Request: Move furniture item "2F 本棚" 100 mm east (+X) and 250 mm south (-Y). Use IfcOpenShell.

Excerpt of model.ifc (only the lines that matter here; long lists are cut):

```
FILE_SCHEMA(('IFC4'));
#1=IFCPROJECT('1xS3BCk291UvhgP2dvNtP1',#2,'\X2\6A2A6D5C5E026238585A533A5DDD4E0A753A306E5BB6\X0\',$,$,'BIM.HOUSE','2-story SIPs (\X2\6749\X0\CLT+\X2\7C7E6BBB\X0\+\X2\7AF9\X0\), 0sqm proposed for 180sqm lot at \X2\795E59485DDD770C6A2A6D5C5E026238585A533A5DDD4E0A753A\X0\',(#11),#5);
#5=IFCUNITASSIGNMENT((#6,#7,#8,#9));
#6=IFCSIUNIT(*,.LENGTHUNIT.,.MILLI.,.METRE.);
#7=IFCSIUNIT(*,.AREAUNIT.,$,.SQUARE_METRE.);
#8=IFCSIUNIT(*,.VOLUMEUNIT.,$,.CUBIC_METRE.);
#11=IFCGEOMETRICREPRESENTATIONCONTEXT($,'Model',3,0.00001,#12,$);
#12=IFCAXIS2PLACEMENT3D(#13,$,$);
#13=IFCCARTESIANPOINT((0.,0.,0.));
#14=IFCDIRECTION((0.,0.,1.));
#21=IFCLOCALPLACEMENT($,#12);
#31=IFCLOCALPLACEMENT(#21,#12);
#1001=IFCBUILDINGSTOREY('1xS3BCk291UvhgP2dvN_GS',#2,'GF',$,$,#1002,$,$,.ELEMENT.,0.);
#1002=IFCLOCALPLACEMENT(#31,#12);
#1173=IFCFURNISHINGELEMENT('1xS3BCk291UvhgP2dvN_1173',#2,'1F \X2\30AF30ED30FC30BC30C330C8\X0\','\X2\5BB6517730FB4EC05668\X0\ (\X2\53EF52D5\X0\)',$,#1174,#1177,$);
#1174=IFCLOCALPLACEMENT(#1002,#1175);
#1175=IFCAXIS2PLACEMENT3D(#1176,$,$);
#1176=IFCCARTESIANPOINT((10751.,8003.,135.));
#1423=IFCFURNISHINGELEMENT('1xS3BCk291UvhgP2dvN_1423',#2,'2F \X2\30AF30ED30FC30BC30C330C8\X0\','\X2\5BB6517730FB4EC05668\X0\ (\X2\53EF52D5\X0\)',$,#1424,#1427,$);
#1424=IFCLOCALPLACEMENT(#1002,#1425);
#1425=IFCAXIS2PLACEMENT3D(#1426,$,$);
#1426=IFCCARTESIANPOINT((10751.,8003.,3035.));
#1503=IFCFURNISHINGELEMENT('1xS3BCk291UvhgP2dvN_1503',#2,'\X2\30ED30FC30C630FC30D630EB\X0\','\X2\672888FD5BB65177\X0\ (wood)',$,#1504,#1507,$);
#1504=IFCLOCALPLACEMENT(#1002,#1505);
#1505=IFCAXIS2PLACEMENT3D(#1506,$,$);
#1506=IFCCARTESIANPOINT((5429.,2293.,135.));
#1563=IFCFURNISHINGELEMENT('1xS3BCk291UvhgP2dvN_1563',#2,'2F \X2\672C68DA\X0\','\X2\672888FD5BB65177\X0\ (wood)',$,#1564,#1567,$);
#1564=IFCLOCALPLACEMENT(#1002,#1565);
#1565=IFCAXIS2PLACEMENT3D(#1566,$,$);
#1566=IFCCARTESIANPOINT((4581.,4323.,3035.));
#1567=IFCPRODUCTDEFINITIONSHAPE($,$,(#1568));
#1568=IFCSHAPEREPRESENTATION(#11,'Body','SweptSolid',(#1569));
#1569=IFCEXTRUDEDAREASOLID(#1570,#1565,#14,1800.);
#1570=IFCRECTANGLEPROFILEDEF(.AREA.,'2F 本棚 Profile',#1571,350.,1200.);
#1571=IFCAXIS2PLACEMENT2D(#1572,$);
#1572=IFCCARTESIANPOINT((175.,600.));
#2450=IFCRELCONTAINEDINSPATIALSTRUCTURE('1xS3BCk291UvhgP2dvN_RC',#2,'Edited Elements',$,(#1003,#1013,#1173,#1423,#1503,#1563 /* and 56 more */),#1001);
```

```python
import ifcopenshell
import ifcopenshell.api.geometry
import ifcopenshell.util.placement
import ifcopenshell.util.unit

model = ifcopenshell.open("model.ifc")
unit_scale = ifcopenshell.util.unit.calculate_unit_scale(model)

item = model.by_guid("1xS3BCk291UvhgP2dvN_1563")
matrix = ifcopenshell.util.placement.get_local_placement(item.ObjectPlacement)
matrix[0, 3] += 0.1 / unit_scale
matrix[1, 3] -= 0.25 / unit_scale
ifcopenshell.api.geometry.edit_object_placement(model, product=item, matrix=matrix, is_si=False)

print(ifcopenshell.util.placement.get_local_placement(item.ObjectPlacement).round(3) + 0.0)

model.write("model_rev.ifc")
```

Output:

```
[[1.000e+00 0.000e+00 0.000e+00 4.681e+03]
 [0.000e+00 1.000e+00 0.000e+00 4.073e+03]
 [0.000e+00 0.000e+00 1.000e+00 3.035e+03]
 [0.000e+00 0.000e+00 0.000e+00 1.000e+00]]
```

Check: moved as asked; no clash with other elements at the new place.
